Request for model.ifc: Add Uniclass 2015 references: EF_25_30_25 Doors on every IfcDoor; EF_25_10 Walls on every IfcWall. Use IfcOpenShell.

First a look at what the model holds.

```python
import ifcopenshell

model = ifcopenshell.open("model.ifc")
print(model.schema)
print("classifications:", [c.Name for c in model.by_type("IfcClassification")])
for ifc_class in ("IfcDoor", "IfcRoof", "IfcStair", "IfcWall", "IfcWindow"):
    print(ifc_class, len(model.by_type(ifc_class)))
```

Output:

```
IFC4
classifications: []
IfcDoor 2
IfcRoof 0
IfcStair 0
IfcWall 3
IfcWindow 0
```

```python
import ifcopenshell
import ifcopenshell.api.classification

model = ifcopenshell.open("model.ifc")

system = ifcopenshell.api.classification.add_classification(model, classification="Uniclass 2015")

codes = {
    "IfcDoor": ("EF_25_30_25", "Doors"),
    "IfcWall": ("EF_25_10", "Walls"),
}
for ifc_class, (code, name) in codes.items():
    products = model.by_type(ifc_class)
    ifcopenshell.api.classification.add_reference(
        model, products=products, classification=system, identification=code, name=name
    )
    print(code, len(products))

model.write("model-out.ifc")
```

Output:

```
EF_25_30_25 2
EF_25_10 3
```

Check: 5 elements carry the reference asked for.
